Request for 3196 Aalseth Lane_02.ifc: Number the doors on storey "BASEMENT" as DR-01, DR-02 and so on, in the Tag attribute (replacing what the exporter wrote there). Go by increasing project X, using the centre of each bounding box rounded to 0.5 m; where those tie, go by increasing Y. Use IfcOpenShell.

First a look at what the model holds.

```python
import ifcopenshell
import ifcopenshell.util.element
import ifcopenshell.util.placement

model = ifcopenshell.open("3196 Aalseth Lane_02.ifc")
print(model.schema)
storey = next(s for s in model.by_type("IfcBuildingStorey") if s.Name == "BASEMENT")
doors = [e for e in ifcopenshell.util.element.get_decomposition(storey) if e.is_a("IfcDoor")]
for e in sorted(doors, key=lambda e: e.id()):
    origin = ifcopenshell.util.placement.get_local_placement(e.ObjectPlacement)[:3, 3]
    print(e.id(), e.Tag, e.Name, origin.round(2) + 0.0, sep=" | ")
```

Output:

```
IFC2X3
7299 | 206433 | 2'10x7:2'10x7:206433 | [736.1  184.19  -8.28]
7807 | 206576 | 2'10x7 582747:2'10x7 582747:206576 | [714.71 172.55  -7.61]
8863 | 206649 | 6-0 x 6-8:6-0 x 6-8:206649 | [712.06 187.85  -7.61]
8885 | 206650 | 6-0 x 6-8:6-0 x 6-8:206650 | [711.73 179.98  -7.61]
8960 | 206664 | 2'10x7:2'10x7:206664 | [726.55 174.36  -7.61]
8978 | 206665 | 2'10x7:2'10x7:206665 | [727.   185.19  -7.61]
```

```python
import ifcopenshell
import ifcopenshell.geom
import ifcopenshell.util.element
import ifcopenshell.util.shape

model = ifcopenshell.open("3196 Aalseth Lane_02.ifc")
settings = ifcopenshell.geom.settings()
settings.set("use-world-coords", True)


def centre(element):
    shape = ifcopenshell.geom.create_shape(settings, element)
    return ifcopenshell.util.shape.get_bbox_centroid(shape.geometry)


storey = next(s for s in model.by_type("IfcBuildingStorey") if s.Name == "BASEMENT")
doors = [e for e in ifcopenshell.util.element.get_decomposition(storey) if e.is_a("IfcDoor")]

# Insertion points can sit at a corner or the storey origin, so sort by the geometry (in metres).
centres = {e: centre(e) for e in doors}
doors.sort(key=lambda e: (round(centres[e][0] / 0.5), centres[e][1]))

for i, e in enumerate(doors, start=1):
    number = f"DR-{i:02d}"
    e.Tag = number
    print(e.id(), number)

model.write("3196 Aalseth Lane_02_rev.ifc")
```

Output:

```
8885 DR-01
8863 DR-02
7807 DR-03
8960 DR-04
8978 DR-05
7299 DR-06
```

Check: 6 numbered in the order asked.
